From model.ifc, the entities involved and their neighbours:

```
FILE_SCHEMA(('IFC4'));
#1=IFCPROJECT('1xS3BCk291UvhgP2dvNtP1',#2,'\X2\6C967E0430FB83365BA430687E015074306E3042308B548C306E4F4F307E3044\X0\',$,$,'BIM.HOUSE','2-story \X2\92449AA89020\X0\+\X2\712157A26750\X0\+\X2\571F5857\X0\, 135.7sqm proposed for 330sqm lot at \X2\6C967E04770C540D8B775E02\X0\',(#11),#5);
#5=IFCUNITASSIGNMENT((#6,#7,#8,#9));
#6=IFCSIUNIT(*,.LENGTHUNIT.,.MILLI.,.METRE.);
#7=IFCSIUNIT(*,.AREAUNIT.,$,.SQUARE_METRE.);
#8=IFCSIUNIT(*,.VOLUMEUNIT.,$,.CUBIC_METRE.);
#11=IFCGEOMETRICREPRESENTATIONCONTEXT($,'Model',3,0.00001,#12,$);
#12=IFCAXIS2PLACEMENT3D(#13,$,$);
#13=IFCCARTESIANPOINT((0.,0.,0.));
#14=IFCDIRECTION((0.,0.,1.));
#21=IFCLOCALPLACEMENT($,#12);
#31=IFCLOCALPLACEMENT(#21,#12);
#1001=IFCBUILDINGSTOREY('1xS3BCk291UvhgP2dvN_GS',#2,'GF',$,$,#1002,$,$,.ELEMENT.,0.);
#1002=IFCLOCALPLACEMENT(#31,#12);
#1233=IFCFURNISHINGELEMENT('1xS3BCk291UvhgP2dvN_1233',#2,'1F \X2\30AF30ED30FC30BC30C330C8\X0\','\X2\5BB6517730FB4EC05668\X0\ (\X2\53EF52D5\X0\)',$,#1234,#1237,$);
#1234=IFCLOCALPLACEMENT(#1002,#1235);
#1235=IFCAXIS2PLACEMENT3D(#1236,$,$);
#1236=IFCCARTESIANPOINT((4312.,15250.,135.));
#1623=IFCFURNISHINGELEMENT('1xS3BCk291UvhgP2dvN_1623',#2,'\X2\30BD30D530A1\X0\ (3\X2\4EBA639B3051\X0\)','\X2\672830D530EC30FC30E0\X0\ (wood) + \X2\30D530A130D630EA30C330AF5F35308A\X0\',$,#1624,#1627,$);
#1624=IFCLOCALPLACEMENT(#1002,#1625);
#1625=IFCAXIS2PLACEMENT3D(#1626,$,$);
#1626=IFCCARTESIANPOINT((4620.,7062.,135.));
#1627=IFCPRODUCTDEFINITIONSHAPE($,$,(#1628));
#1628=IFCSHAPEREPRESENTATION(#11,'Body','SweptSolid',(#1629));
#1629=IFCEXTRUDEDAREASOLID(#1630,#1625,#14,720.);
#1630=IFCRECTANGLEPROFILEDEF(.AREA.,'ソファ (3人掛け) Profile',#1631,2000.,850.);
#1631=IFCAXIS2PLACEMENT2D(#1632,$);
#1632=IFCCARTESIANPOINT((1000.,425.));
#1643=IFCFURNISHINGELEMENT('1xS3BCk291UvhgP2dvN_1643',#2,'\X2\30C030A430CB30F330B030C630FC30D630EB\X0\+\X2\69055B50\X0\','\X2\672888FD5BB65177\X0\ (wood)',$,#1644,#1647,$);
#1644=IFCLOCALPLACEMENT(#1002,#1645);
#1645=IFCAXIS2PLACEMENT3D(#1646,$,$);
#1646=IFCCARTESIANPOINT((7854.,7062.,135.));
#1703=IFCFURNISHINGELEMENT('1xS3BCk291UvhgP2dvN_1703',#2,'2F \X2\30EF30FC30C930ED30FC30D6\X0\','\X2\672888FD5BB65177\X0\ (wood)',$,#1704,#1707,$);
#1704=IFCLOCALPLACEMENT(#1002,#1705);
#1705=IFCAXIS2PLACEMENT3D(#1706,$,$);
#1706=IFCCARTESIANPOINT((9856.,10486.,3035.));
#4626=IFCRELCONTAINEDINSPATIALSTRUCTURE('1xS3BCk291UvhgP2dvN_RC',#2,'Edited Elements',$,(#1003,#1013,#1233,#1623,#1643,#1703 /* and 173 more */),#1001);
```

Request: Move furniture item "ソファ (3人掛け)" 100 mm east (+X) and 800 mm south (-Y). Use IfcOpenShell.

```python
import ifcopenshell
import ifcopenshell.api.geometry
import ifcopenshell.util.placement
import ifcopenshell.util.unit

model = ifcopenshell.open("model.ifc")
unit_scale = ifcopenshell.util.unit.calculate_unit_scale(model)

item = model.by_guid("1xS3BCk291UvhgP2dvN_1623")
matrix = ifcopenshell.util.placement.get_local_placement(item.ObjectPlacement)
matrix[0, 3] += 0.1 / unit_scale
matrix[1, 3] -= 0.8 / unit_scale
ifcopenshell.api.geometry.edit_object_placement(model, product=item, matrix=matrix, is_si=False)

print(ifcopenshell.util.placement.get_local_placement(item.ObjectPlacement).round(3) + 0.0)

model.write("model_updated.ifc")
```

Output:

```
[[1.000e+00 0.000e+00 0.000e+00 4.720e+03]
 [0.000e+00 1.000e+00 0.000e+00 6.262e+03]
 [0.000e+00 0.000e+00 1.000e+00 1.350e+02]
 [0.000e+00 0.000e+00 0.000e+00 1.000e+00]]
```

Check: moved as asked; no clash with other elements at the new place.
